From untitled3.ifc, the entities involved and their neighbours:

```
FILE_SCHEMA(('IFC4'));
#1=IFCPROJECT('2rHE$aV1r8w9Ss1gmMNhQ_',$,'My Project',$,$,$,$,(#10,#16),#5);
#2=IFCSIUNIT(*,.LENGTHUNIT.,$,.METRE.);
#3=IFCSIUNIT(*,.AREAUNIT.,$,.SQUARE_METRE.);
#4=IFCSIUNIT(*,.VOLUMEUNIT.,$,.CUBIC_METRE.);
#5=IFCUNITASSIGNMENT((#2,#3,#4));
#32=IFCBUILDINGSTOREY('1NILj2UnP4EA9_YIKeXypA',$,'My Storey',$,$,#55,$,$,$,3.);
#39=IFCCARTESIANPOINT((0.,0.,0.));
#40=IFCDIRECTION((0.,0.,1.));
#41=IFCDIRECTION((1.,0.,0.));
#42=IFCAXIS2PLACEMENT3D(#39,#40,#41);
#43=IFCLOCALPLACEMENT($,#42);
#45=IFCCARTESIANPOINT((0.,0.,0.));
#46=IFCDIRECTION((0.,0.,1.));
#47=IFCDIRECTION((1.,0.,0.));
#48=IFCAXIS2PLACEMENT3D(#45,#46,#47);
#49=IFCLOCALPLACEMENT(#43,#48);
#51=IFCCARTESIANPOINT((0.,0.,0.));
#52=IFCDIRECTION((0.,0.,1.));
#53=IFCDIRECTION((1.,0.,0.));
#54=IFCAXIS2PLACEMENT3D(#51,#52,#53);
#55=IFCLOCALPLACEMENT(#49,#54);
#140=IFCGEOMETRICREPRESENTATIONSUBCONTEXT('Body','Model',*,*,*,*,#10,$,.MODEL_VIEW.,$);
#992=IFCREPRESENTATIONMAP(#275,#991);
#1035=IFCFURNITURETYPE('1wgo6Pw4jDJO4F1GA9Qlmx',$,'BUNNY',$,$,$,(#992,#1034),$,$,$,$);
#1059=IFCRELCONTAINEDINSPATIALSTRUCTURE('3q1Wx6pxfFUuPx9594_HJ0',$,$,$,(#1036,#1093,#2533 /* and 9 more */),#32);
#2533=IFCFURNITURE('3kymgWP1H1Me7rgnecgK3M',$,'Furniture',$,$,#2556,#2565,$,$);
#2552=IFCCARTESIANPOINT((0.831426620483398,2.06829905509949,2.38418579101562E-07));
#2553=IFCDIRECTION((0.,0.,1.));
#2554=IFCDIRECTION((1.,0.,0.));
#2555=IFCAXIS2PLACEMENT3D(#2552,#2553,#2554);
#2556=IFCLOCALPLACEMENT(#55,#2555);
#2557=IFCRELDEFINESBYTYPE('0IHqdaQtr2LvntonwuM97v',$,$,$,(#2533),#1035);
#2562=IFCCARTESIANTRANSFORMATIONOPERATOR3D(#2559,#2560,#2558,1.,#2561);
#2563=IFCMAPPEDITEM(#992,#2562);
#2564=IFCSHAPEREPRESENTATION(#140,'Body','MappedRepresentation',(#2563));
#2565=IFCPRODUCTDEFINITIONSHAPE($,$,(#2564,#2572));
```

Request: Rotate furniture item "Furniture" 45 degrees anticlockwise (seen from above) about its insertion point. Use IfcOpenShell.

```python
import ifcopenshell
import ifcopenshell.api.geometry
import ifcopenshell.util.placement

model = ifcopenshell.open("untitled3.ifc")

item = model.by_guid("3kymgWP1H1Me7rgnecgK3M")
matrix = ifcopenshell.util.placement.get_local_placement(item.ObjectPlacement)
matrix = matrix @ ifcopenshell.util.placement.rotation(45, "Z")
ifcopenshell.api.geometry.edit_object_placement(model, product=item, matrix=matrix, is_si=False)

print(ifcopenshell.util.placement.get_local_placement(item.ObjectPlacement).round(3) + 0.0)

model.write("untitled3_updated.ifc")
```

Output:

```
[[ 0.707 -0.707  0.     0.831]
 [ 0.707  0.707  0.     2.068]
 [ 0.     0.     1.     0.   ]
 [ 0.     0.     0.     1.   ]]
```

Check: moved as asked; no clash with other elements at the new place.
